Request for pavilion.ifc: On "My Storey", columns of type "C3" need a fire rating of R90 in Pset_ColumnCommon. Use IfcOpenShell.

First a look at what the model holds.

```python
import ifcopenshell
import ifcopenshell.util.element

model = ifcopenshell.open("pavilion.ifc")
print(model.schema)
storey = next(s for s in model.by_type("IfcBuildingStorey") if s.Name == "My Storey")
columns = [e for e in ifcopenshell.util.element.get_decomposition(storey) if e.is_a("IfcColumn")]
seen = {}
for e in columns:
    element_type = ifcopenshell.util.element.get_type(e)
    key = (element_type.Name if element_type != e and element_type else None, ifcopenshell.util.element.get_pset(e, "Pset_ColumnCommon", "FireRating"))
    seen[key] = seen.get(key, 0) + 1
for (name, value), count in sorted(seen.items(), key=str):
    print(count, "x", name, "|", value)
```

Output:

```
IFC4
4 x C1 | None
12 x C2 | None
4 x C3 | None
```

```python
import ifcopenshell
import ifcopenshell.api.pset
import ifcopenshell.util.element

model = ifcopenshell.open("pavilion.ifc")

storey = next(s for s in model.by_type("IfcBuildingStorey") if s.Name == "My Storey")
columns = [e for e in ifcopenshell.util.element.get_decomposition(storey) if e.is_a("IfcColumn")]

count = 0
for e in columns:
    element_type = ifcopenshell.util.element.get_type(e)
    if element_type in (None, e) or element_type.Name != "C3":
        continue
    # add_pset returns the element's existing set when there is one.
    pset = ifcopenshell.api.pset.add_pset(model, product=e, name="Pset_ColumnCommon")
    ifcopenshell.api.pset.edit_pset(model, pset=pset, properties={"FireRating": "R90"})
    count += 1

print(count, "columns updated")

model.write("pavilion_v2.ifc")
```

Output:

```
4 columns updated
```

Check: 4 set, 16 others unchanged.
